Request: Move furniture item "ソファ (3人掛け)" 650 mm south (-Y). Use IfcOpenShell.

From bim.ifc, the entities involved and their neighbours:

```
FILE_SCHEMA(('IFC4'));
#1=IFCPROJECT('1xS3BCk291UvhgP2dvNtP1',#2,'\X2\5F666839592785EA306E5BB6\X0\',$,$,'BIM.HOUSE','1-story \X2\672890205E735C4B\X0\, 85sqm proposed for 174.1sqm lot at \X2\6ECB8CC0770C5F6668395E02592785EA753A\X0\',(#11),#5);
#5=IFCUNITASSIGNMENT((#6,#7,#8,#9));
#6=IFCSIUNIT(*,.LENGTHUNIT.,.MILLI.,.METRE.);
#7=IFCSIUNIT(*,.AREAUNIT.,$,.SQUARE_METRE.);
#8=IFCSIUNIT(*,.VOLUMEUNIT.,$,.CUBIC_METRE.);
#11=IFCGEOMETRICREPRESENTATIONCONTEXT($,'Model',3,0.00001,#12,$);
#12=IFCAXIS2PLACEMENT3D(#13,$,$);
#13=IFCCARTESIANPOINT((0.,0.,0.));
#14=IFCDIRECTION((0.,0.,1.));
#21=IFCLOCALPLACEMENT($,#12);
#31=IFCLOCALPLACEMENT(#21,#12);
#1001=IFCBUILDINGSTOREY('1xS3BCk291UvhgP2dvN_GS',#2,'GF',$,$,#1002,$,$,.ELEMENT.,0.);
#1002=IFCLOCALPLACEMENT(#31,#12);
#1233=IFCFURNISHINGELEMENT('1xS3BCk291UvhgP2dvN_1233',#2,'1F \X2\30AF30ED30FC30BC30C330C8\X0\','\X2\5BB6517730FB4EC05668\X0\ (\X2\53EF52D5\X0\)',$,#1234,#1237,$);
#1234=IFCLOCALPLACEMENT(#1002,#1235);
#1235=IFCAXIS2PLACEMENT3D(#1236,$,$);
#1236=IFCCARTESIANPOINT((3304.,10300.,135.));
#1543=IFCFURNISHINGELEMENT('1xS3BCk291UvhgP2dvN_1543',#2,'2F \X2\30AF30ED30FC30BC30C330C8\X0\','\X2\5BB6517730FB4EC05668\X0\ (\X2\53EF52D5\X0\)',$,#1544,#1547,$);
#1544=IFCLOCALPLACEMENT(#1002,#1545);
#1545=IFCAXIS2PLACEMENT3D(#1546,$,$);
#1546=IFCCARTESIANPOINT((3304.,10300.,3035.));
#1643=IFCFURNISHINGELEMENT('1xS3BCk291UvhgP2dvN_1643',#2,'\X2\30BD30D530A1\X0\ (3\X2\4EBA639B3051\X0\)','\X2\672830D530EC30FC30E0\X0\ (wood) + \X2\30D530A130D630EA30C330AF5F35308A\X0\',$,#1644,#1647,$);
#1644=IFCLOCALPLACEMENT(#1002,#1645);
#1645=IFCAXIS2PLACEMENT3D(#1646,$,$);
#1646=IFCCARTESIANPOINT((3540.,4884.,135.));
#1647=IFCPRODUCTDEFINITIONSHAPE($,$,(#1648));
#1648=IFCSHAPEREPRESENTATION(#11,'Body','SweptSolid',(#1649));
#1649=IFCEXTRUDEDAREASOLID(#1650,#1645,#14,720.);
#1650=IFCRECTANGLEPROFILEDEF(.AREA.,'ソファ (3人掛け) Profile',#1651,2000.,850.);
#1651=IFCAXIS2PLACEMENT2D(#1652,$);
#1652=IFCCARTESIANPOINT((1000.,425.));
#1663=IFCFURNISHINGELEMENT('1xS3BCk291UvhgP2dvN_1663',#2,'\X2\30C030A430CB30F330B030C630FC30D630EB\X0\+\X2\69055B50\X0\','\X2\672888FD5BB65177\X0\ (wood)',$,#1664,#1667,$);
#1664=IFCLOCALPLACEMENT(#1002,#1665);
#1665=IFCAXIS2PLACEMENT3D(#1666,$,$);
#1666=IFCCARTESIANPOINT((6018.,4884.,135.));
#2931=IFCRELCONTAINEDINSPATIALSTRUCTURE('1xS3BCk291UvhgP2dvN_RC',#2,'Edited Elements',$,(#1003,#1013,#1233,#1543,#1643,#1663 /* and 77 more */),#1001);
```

```python
import ifcopenshell
import ifcopenshell.api.geometry
import ifcopenshell.util.placement

model = ifcopenshell.open("bim.ifc")

item = model.by_guid("1xS3BCk291UvhgP2dvN_1643")
matrix = ifcopenshell.util.placement.get_local_placement(item.ObjectPlacement)
matrix[1, 3] -= 650.0
ifcopenshell.api.geometry.edit_object_placement(model, product=item, matrix=matrix, is_si=False)

print(ifcopenshell.util.placement.get_local_placement(item.ObjectPlacement).round(3) + 0.0)

model.write("bim_edited.ifc")
```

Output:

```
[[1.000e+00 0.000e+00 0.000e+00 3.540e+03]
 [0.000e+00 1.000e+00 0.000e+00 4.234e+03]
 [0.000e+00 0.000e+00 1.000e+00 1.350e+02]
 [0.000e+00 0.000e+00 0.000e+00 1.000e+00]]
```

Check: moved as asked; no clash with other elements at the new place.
